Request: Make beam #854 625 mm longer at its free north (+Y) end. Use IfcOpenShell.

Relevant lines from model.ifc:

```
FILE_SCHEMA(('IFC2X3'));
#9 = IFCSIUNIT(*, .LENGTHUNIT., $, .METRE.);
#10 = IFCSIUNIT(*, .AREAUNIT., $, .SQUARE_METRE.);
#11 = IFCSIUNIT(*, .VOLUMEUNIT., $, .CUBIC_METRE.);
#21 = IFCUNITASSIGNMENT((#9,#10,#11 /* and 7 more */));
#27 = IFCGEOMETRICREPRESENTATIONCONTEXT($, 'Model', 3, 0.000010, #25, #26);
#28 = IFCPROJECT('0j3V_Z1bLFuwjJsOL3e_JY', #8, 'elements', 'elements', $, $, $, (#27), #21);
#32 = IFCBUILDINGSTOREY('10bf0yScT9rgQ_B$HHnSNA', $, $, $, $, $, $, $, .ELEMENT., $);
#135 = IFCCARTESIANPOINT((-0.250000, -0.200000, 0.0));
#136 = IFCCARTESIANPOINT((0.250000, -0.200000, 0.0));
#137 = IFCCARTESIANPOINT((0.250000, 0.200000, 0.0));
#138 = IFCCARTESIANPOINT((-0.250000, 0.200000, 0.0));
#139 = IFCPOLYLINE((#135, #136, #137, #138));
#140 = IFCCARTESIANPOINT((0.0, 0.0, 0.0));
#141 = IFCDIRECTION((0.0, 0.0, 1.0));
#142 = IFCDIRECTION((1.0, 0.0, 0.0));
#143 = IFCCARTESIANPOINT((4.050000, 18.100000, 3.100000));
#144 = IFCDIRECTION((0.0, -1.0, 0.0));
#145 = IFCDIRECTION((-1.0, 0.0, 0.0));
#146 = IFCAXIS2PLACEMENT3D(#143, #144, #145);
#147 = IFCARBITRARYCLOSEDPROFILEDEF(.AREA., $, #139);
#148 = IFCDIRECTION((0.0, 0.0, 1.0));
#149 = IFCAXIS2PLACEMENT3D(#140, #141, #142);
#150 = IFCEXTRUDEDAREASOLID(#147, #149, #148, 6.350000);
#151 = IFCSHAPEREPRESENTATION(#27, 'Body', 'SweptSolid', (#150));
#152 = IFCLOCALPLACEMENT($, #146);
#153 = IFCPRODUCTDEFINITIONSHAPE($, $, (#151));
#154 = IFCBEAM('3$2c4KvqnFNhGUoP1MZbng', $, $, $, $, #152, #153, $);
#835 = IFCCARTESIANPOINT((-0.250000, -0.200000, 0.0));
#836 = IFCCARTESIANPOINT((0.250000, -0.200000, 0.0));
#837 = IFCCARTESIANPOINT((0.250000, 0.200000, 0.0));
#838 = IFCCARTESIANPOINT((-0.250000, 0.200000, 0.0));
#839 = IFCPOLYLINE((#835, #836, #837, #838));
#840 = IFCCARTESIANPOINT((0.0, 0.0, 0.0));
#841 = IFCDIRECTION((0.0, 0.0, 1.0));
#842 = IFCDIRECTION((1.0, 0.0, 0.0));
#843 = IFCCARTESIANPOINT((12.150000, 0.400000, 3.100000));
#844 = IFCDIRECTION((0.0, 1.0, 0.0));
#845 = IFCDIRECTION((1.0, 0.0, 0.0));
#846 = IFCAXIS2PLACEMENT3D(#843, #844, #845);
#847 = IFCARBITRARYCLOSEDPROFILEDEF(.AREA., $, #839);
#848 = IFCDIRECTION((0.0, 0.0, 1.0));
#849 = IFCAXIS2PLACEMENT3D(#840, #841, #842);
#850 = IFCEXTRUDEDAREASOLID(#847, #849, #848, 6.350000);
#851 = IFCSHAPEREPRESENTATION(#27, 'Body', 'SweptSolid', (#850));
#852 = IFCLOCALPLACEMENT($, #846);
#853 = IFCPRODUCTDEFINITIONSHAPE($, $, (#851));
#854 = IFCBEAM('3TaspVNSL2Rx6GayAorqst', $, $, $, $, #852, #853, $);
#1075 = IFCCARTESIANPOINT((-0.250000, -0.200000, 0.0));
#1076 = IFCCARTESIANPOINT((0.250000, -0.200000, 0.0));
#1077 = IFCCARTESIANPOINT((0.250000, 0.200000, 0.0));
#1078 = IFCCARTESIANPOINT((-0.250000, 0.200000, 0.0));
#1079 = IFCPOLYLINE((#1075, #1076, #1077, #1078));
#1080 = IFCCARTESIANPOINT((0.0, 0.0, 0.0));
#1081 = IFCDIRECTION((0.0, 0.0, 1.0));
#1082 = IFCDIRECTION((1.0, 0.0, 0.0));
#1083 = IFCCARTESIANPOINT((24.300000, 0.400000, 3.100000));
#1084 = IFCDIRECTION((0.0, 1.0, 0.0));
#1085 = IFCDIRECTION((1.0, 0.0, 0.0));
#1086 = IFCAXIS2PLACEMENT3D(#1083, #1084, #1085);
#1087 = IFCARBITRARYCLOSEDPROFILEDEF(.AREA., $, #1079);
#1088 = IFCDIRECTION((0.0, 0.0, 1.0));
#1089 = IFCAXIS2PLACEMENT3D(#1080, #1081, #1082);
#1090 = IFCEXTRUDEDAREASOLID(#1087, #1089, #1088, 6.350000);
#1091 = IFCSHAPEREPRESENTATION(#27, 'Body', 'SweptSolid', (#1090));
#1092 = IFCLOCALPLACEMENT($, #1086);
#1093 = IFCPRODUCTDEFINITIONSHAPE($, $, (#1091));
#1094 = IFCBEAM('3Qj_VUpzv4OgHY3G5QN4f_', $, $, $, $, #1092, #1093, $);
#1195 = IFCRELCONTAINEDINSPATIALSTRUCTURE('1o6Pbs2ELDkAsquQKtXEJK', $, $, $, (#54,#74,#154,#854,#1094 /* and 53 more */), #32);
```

```python
import ifcopenshell

model = ifcopenshell.open("model.ifc")

member = model.by_guid("3TaspVNSL2Rx6GayAorqst")
change = 0.625

# The extrusion runs towards the end named, so only its depth changes.
body = next(r for r in member.Representation.Representations if r.RepresentationIdentifier == "Body")
solid = body.Items[0]
old_length = solid.Depth
solid.Depth += change

print(f"length {old_length:g} -> {solid.Depth:g}")

model.write("model-out.ifc")
```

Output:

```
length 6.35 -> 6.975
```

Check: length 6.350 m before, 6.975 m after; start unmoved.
